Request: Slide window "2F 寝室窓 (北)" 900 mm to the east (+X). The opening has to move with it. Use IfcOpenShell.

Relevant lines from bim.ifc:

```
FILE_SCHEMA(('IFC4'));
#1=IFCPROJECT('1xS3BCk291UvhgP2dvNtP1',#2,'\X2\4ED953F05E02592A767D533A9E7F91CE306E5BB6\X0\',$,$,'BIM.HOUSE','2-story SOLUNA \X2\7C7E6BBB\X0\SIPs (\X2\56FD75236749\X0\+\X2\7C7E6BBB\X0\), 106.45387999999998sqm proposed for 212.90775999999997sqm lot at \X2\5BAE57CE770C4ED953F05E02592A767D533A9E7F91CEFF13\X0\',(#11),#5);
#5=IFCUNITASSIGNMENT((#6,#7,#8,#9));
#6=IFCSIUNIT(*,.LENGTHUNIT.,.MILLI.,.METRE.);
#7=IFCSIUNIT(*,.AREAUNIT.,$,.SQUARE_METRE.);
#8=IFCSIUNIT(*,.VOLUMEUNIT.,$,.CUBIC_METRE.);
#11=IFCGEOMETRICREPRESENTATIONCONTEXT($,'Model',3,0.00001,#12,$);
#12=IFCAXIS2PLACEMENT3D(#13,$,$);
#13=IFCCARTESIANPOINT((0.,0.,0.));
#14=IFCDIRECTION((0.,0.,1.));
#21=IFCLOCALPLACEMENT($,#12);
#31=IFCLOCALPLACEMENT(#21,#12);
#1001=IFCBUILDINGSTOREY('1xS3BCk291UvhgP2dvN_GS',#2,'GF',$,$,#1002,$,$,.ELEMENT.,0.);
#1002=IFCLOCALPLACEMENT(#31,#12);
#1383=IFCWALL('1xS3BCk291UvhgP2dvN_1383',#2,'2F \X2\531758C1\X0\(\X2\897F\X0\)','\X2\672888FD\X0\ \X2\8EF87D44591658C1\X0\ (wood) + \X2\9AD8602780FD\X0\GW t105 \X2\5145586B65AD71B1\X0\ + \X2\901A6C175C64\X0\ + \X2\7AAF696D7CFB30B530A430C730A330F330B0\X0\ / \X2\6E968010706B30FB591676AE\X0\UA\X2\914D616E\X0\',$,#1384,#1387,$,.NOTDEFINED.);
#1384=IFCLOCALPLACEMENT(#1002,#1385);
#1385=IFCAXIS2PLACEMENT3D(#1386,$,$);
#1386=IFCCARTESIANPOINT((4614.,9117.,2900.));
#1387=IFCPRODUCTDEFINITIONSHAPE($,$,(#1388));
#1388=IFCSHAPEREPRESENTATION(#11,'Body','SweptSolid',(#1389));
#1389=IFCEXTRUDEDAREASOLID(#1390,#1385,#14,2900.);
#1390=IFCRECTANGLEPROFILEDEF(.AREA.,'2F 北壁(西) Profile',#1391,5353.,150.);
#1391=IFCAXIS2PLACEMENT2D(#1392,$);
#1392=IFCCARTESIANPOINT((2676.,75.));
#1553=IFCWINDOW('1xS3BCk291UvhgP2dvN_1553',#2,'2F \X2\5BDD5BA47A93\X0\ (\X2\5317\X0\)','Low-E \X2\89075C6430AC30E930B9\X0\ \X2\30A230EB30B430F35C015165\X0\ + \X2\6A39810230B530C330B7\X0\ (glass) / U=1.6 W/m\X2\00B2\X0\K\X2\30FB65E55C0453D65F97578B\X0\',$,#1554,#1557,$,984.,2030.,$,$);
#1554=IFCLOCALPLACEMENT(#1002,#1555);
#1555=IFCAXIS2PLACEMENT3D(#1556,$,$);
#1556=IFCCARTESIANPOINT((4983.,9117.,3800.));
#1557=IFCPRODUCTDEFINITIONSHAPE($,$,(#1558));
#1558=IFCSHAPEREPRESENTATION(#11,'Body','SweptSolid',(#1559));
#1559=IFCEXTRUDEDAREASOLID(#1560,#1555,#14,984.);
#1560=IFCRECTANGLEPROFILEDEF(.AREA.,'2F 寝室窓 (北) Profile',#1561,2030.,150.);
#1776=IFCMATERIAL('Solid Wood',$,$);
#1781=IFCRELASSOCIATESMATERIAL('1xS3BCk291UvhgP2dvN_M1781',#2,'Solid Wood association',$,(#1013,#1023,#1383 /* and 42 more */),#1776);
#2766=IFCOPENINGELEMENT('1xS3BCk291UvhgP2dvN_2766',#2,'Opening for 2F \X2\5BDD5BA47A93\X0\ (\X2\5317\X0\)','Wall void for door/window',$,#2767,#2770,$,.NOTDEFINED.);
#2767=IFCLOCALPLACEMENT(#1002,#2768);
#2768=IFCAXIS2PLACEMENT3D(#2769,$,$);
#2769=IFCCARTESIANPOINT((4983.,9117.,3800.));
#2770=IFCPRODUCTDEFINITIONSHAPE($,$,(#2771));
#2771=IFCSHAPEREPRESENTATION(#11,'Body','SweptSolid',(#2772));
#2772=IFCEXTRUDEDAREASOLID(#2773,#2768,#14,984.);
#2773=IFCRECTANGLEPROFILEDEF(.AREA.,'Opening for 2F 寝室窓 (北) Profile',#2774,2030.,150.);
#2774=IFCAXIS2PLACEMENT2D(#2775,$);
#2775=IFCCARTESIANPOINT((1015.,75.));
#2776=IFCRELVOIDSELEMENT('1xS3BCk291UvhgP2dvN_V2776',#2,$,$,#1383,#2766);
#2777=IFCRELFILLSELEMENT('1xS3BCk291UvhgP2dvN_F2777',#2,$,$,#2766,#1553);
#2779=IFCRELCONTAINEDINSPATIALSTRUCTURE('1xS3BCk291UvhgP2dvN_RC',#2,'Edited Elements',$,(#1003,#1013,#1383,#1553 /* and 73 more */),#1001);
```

```python
import ifcopenshell
import ifcopenshell.api.geometry
import ifcopenshell.util.placement

model = ifcopenshell.open("bim.ifc")

window = model.by_id(1553)
opening = window.FillsVoids[0].RelatingOpeningElement
wall = opening.VoidsElements[0].RelatingBuildingElement

wall_matrix = ifcopenshell.util.placement.get_local_placement(wall.ObjectPlacement)
shift = wall_matrix[:3, 0] * 900.0
before = ifcopenshell.util.placement.get_local_placement(window.ObjectPlacement)[:3, 3].copy()

# The window is not placed relative to its opening, so move both.
for product in (opening, window):
    matrix = ifcopenshell.util.placement.get_local_placement(product.ObjectPlacement)
    matrix[:3, 3] += shift
    ifcopenshell.api.geometry.edit_object_placement(model, product=product, matrix=matrix, is_si=False)

after = ifcopenshell.util.placement.get_local_placement(window.ObjectPlacement)[:3, 3]
print("window moved by", (after - before).round(3) + 0.0)

model.write("bim_rev.ifc")
```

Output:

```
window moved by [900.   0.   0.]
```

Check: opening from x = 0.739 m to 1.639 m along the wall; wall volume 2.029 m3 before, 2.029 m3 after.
